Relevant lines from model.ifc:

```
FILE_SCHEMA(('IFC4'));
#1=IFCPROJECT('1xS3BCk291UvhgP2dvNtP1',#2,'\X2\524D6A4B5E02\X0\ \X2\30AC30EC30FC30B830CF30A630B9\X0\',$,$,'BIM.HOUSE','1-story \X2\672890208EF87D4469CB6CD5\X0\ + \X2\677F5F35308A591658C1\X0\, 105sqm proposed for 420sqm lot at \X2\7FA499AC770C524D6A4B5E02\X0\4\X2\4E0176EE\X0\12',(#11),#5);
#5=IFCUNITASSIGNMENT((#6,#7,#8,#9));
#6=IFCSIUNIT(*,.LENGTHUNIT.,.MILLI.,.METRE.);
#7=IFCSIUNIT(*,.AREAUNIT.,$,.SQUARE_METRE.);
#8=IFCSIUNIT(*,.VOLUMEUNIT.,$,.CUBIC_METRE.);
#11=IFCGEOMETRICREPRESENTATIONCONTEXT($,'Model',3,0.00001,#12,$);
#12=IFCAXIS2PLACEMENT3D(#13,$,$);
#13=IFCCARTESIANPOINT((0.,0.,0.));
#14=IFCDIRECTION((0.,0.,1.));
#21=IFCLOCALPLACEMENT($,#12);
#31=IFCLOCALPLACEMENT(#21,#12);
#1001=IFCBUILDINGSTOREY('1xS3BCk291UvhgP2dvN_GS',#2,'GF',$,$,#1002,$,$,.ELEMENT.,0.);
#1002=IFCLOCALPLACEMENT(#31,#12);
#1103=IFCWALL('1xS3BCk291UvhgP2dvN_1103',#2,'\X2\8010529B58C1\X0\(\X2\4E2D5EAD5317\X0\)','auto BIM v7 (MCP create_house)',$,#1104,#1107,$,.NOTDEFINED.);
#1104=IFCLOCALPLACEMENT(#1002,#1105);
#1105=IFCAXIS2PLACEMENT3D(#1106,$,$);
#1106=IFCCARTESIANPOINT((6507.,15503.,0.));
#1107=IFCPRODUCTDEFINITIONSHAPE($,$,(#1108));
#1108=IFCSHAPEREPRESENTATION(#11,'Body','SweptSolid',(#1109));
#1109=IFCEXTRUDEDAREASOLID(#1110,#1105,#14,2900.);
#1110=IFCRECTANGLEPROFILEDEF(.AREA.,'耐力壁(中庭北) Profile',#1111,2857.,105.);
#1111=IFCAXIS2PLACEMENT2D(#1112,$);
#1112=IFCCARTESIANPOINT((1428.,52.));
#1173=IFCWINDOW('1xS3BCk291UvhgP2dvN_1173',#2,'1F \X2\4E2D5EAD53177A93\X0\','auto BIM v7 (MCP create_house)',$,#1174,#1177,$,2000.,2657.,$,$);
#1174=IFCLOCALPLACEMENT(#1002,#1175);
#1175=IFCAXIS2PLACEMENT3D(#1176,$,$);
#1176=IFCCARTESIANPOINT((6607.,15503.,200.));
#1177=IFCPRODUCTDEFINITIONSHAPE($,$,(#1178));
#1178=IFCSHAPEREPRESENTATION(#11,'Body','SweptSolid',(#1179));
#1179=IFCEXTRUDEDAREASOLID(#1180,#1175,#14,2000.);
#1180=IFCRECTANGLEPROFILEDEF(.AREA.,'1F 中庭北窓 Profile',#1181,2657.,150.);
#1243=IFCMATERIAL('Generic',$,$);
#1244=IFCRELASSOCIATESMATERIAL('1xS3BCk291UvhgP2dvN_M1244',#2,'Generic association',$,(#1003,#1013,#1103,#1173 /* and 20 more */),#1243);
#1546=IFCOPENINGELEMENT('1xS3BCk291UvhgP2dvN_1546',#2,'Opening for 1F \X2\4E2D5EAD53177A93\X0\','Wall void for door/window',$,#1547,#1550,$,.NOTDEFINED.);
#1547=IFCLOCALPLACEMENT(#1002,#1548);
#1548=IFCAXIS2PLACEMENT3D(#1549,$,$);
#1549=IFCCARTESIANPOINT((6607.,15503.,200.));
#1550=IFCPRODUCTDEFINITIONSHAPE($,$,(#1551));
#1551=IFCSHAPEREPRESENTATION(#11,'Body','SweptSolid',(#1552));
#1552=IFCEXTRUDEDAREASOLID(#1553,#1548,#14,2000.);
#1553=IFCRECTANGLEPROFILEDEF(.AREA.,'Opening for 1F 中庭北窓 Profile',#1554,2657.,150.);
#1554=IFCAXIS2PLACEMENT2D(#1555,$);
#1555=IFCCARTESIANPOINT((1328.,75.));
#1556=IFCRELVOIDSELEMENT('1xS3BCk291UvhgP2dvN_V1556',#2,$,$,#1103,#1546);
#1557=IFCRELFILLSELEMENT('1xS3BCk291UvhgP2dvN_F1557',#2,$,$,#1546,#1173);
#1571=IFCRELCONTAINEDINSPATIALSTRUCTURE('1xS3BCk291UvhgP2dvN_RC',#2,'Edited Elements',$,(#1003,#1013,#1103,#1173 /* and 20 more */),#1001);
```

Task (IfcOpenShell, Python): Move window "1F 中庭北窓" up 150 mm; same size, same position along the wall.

```python
import numpy as np
import ifcopenshell
import ifcopenshell.api.geometry
import ifcopenshell.util.placement
import ifcopenshell.util.unit

model = ifcopenshell.open("model.ifc")
unit_scale = ifcopenshell.util.unit.calculate_unit_scale(model)

window = model.by_guid("1xS3BCk291UvhgP2dvN_1173")
opening = window.FillsVoids[0].RelatingOpeningElement
dz = 0.15 / unit_scale

shift = np.array([0.0, 0.0, dz])
# The window is not placed relative to its opening, so move both.
for product in (opening, window):
    matrix = ifcopenshell.util.placement.get_local_placement(product.ObjectPlacement)
    matrix[:3, 3] += shift
    ifcopenshell.api.geometry.edit_object_placement(model, product=product, matrix=matrix, is_si=False)

print(f"moved by {dz * unit_scale:+.3f} m")

model.write("model_updated.ifc")
```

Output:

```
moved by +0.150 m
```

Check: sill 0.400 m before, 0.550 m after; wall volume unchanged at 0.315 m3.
